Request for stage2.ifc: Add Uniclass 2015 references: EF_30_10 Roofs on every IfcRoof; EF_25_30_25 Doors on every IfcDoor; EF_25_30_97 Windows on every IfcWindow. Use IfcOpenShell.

First a look at what the model holds.

```python
import ifcopenshell

model = ifcopenshell.open("stage2.ifc")
print(model.schema)
print("classifications:", [c.Name for c in model.by_type("IfcClassification")])
for ifc_class in ("IfcDoor", "IfcRoof", "IfcStair", "IfcWall", "IfcWindow"):
    print(ifc_class, len(model.by_type(ifc_class)))
```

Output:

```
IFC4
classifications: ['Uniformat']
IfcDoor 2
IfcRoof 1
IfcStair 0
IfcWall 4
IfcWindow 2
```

```python
import ifcopenshell
import ifcopenshell.api.classification

model = ifcopenshell.open("stage2.ifc")

system = ifcopenshell.api.classification.add_classification(model, classification="Uniclass 2015")

codes = {
    "IfcRoof": ("EF_30_10", "Roofs"),
    "IfcDoor": ("EF_25_30_25", "Doors"),
    "IfcWindow": ("EF_25_30_97", "Windows"),
}
for ifc_class, (code, name) in codes.items():
    products = model.by_type(ifc_class)
    ifcopenshell.api.classification.add_reference(
        model, products=products, classification=system, identification=code, name=name
    )
    print(code, len(products))

model.write("stage2_edited.ifc")
```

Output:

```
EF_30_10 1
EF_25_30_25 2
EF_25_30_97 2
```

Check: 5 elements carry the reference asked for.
